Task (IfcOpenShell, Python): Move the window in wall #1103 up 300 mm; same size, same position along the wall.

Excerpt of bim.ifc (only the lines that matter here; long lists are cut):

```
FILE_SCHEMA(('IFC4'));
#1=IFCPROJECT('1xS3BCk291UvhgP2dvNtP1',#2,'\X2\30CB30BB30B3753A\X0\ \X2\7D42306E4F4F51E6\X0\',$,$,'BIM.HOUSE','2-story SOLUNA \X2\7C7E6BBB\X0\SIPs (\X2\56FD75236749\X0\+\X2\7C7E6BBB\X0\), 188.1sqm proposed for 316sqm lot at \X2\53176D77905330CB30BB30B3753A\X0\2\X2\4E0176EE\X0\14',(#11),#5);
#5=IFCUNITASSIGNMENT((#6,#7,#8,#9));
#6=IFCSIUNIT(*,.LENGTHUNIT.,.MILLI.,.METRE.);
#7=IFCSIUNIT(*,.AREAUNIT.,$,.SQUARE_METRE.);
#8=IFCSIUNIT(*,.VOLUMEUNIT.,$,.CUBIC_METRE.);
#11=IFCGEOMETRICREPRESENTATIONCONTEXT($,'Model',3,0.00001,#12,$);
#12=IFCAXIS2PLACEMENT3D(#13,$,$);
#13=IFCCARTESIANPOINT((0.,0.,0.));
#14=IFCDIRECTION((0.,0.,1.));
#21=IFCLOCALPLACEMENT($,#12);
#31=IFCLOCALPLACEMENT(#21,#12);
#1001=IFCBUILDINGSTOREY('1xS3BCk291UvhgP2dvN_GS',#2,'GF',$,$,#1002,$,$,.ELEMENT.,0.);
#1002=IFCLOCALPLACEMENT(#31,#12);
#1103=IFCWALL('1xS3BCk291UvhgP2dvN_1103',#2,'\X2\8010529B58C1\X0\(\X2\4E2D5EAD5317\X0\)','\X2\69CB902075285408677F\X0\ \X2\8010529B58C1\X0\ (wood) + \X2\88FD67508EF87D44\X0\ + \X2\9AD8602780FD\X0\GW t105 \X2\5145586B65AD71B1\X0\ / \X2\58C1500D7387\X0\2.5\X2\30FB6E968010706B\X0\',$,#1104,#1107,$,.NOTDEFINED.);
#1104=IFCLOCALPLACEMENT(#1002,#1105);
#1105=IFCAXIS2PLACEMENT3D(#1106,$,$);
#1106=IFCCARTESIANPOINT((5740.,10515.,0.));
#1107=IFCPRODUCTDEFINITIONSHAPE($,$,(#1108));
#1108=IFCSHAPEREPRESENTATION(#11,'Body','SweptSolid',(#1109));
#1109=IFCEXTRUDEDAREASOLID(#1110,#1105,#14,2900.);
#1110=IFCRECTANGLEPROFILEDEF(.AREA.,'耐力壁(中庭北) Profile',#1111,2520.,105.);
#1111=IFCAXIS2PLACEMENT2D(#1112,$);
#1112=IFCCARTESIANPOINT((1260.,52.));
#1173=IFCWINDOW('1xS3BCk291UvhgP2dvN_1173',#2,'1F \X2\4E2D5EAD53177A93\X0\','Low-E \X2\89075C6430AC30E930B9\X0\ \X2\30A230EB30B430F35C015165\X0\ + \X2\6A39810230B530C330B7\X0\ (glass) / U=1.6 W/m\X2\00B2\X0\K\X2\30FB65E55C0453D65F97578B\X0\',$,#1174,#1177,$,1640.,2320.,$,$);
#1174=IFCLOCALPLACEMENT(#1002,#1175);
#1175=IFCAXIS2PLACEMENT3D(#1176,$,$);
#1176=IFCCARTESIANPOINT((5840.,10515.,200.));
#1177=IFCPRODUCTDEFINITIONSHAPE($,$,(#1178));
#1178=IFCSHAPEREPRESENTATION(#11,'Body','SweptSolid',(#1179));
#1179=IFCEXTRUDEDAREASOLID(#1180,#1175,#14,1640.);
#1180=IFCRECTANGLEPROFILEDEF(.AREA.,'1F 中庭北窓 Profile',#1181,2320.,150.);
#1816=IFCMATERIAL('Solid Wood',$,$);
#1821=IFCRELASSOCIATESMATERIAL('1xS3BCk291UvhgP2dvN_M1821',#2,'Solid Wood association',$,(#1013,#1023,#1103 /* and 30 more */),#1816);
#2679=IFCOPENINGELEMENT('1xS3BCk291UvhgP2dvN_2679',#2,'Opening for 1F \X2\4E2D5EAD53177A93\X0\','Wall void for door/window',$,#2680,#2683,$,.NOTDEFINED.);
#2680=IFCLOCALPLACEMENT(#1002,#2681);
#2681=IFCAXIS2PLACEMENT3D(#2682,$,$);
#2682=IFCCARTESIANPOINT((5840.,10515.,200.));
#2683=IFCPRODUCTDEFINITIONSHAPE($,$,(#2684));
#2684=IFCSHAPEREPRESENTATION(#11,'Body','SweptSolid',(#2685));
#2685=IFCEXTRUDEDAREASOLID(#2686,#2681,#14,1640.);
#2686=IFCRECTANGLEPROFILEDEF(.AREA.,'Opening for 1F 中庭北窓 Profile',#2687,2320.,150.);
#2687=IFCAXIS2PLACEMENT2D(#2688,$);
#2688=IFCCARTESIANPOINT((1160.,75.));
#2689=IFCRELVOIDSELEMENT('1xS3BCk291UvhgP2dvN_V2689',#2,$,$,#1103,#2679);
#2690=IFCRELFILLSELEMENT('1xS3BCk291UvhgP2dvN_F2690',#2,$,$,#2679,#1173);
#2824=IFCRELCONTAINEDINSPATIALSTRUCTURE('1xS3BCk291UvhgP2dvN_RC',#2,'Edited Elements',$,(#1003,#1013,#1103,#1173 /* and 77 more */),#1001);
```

```python
import numpy as np
import ifcopenshell
import ifcopenshell.api.geometry
import ifcopenshell.util.placement
import ifcopenshell.util.unit

model = ifcopenshell.open("bim.ifc")
unit_scale = ifcopenshell.util.unit.calculate_unit_scale(model)

window = model.by_id(1173)
opening = window.FillsVoids[0].RelatingOpeningElement
dz = 0.3 / unit_scale

shift = np.array([0.0, 0.0, dz])
# The window is not placed relative to its opening, so move both.
for product in (opening, window):
    matrix = ifcopenshell.util.placement.get_local_placement(product.ObjectPlacement)
    matrix[:3, 3] += shift
    ifcopenshell.api.geometry.edit_object_placement(model, product=product, matrix=matrix, is_si=False)

print(f"moved by {dz * unit_scale:+.3f} m")

model.write("bim_edited.ifc")
```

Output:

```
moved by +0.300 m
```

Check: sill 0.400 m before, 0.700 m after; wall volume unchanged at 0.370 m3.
